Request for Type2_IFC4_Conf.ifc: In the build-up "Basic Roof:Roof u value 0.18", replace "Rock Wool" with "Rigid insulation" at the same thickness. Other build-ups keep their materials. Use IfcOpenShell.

First a look at what the model holds.

```python
import ifcopenshell
import ifcopenshell.util.element

model = ifcopenshell.open("Type2_IFC4_Conf.ifc")
print(model.schema)
for layer_set in model.by_type("IfcMaterialLayerSet"):
    if layer_set.LayerSetName == "Basic Roof:Roof u value 0.18":
        for layer in layer_set.MaterialLayers:
            print(layer.id(), layer.Material and layer.Material.Name, layer.LayerThickness, sep=" | ")
        print(len(ifcopenshell.util.element.get_elements_by_material(model, layer_set)), "elements and types use it")
print(sorted(m.Name for m in model.by_type("IfcMaterial") if m.Name)[:60])
```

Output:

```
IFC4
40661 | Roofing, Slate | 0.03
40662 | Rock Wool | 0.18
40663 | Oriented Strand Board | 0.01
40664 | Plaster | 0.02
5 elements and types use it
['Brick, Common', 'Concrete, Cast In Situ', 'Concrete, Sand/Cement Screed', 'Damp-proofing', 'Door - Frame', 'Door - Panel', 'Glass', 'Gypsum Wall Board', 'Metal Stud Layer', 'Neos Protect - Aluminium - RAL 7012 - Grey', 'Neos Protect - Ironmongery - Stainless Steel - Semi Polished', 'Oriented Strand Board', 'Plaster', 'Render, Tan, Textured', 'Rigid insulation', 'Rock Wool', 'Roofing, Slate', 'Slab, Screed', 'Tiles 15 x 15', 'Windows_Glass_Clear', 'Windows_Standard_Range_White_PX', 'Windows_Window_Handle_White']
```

```python
import ifcopenshell
import ifcopenshell.api.material

model = ifcopenshell.open("Type2_IFC4_Conf.ifc")

layer_set = next(s for s in model.by_type("IfcMaterialLayerSet") if s.LayerSetName == "Basic Roof:Roof u value 0.18")
layer = next(l for l in layer_set.MaterialLayers if l.Material and l.Material.Name == "Rock Wool")
material = next(m for m in model.by_type("IfcMaterial") if m.Name == "Rigid insulation")

# Point this one layer at the other material; renaming the old one would change it everywhere.
ifcopenshell.api.material.edit_layer(model, layer=layer, attributes={"Name": material.Name}, material=material)

print([l.Material.Name if l.Material else None for l in layer_set.MaterialLayers])

model.write("Type2_IFC4_Conf_rev.ifc")
```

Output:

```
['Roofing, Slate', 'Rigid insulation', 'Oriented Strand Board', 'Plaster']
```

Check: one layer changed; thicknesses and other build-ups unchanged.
